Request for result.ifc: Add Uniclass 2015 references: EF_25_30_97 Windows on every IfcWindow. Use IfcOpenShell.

First a look at what the model holds.

```python
import ifcopenshell

model = ifcopenshell.open("result.ifc")
print(model.schema)
print("classifications:", [c.Name for c in model.by_type("IfcClassification")])
for ifc_class in ("IfcDoor", "IfcRoof", "IfcStair", "IfcWall", "IfcWindow"):
    print(ifc_class, len(model.by_type(ifc_class)))
```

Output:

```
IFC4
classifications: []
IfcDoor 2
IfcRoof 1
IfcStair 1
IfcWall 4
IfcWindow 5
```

```python
import ifcopenshell
import ifcopenshell.api.classification

model = ifcopenshell.open("result.ifc")

system = ifcopenshell.api.classification.add_classification(model, classification="Uniclass 2015")

codes = {
    "IfcWindow": ("EF_25_30_97", "Windows"),
}
for ifc_class, (code, name) in codes.items():
    products = model.by_type(ifc_class)
    ifcopenshell.api.classification.add_reference(
        model, products=products, classification=system, identification=code, name=name
    )
    print(code, len(products))

model.write("result_edited.ifc")
```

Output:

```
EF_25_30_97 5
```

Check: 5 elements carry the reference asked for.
